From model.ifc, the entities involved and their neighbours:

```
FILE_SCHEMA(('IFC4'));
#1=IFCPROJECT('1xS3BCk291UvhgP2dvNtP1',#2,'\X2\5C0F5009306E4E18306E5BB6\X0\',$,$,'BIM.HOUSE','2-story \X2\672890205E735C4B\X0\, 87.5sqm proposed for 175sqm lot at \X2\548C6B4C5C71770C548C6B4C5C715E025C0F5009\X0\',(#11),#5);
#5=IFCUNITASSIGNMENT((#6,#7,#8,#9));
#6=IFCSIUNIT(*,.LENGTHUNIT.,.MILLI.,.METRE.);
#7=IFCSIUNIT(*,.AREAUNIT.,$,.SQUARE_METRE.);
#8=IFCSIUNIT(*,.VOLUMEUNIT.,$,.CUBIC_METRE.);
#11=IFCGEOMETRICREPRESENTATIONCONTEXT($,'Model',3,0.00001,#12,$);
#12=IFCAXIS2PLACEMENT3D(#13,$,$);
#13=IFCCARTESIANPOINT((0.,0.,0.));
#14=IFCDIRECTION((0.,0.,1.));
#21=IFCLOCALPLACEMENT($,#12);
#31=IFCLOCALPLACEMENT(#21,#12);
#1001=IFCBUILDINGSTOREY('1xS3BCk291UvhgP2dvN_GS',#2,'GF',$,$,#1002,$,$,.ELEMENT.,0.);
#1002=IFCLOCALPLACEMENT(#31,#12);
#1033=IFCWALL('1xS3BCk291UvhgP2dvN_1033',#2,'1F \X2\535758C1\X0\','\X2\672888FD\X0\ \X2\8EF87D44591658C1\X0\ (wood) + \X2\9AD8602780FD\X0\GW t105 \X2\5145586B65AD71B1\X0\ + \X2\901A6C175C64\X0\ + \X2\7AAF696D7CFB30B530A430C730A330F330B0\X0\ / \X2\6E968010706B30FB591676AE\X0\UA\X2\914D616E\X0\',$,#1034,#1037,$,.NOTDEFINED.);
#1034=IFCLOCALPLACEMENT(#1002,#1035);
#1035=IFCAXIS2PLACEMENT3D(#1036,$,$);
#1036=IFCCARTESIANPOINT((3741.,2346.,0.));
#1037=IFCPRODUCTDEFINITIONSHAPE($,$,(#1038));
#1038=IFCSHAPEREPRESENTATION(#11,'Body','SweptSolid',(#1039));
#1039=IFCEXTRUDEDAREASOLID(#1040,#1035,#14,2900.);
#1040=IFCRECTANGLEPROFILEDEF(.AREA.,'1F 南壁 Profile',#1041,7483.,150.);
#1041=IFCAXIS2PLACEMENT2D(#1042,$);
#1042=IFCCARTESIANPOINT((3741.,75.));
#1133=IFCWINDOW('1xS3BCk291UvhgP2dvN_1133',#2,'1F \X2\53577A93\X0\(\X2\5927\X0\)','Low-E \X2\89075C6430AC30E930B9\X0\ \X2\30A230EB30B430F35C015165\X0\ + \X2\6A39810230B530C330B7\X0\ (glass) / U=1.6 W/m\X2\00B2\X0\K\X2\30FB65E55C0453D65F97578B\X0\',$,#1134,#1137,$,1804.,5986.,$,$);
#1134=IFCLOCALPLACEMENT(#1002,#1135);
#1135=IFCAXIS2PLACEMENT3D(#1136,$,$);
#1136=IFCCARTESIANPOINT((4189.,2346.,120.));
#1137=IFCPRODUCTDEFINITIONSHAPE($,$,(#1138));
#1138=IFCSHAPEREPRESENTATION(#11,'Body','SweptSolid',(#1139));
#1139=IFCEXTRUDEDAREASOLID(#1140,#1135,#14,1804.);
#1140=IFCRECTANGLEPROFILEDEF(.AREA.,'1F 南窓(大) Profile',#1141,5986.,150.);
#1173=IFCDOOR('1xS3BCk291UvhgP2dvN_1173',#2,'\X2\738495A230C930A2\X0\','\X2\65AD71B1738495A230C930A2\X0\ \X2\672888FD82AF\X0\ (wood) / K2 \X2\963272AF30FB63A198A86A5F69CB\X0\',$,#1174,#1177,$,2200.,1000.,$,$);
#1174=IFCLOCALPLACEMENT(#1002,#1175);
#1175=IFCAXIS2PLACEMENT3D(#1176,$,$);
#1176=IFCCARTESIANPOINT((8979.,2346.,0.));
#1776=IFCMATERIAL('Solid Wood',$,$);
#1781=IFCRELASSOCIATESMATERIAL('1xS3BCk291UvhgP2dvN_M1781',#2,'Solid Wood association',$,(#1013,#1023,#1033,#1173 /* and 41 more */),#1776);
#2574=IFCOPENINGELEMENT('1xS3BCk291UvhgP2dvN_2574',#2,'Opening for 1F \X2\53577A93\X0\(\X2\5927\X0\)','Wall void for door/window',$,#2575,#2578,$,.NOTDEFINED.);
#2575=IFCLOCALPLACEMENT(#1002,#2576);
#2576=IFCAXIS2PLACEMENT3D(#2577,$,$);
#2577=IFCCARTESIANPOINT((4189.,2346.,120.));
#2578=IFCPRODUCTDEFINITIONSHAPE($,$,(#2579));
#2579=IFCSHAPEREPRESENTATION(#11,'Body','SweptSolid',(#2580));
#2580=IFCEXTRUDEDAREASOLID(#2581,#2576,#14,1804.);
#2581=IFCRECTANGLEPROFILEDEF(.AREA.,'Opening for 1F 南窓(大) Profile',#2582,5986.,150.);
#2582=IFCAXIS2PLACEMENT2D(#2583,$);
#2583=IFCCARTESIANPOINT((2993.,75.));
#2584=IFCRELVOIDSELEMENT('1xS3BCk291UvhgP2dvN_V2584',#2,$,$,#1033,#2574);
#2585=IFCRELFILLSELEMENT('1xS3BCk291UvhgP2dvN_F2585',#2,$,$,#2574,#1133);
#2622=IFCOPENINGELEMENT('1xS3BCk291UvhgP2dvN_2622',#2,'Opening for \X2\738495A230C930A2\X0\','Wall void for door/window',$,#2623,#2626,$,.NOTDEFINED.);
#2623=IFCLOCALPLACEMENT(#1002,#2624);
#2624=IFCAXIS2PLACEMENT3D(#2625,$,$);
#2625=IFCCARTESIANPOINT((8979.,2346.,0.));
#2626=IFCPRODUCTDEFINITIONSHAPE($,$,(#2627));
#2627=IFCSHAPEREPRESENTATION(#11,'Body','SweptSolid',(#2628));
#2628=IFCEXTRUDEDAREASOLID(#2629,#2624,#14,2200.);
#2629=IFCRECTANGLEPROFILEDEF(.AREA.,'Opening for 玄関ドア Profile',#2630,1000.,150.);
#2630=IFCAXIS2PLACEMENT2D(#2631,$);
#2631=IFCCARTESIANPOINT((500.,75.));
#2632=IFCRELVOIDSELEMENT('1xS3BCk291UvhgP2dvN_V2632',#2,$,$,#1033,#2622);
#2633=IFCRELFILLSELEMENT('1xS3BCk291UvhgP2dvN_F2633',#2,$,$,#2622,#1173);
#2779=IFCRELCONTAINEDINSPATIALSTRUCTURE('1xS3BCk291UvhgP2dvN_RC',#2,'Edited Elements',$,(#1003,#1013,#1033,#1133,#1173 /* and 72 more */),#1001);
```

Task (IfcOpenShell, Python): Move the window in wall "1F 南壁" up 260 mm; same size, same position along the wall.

```python
import numpy as np
import ifcopenshell
import ifcopenshell.api.geometry
import ifcopenshell.util.placement
import ifcopenshell.util.unit

model = ifcopenshell.open("model.ifc")
unit_scale = ifcopenshell.util.unit.calculate_unit_scale(model)

window = model.by_guid("1xS3BCk291UvhgP2dvN_1133")
opening = window.FillsVoids[0].RelatingOpeningElement
dz = 260.0

shift = np.array([0.0, 0.0, dz])
# The window is not placed relative to its opening, so move both.
for product in (opening, window):
    matrix = ifcopenshell.util.placement.get_local_placement(product.ObjectPlacement)
    matrix[:3, 3] += shift
    ifcopenshell.api.geometry.edit_object_placement(model, product=product, matrix=matrix, is_si=False)

print(f"moved by {dz * unit_scale:+.3f} m")

model.write("model_updated.ifc")
```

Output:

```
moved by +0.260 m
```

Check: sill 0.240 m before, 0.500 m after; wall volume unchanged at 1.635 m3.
